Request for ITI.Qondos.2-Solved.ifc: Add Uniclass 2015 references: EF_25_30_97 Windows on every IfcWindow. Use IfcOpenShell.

First a look at what the model holds.

```python
import ifcopenshell

model = ifcopenshell.open("ITI.Qondos.2-Solved.ifc")
print(model.schema)
print("classifications:", [c.Name for c in model.by_type("IfcClassification")])
for ifc_class in ("IfcDoor", "IfcRoof", "IfcStair", "IfcWall", "IfcWindow"):
    print(ifc_class, len(model.by_type(ifc_class)))
```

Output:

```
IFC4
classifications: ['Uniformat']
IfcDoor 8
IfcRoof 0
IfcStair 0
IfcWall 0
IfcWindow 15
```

```python
import ifcopenshell
import ifcopenshell.api.classification

model = ifcopenshell.open("ITI.Qondos.2-Solved.ifc")

system = ifcopenshell.api.classification.add_classification(model, classification="Uniclass 2015")

codes = {
    "IfcWindow": ("EF_25_30_97", "Windows"),
}
for ifc_class, (code, name) in codes.items():
    products = model.by_type(ifc_class)
    ifcopenshell.api.classification.add_reference(
        model, products=products, classification=system, identification=code, name=name
    )
    print(code, len(products))

model.write("ITI.Qondos.2-Solved_v2.ifc")
```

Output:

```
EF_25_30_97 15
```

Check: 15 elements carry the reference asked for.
